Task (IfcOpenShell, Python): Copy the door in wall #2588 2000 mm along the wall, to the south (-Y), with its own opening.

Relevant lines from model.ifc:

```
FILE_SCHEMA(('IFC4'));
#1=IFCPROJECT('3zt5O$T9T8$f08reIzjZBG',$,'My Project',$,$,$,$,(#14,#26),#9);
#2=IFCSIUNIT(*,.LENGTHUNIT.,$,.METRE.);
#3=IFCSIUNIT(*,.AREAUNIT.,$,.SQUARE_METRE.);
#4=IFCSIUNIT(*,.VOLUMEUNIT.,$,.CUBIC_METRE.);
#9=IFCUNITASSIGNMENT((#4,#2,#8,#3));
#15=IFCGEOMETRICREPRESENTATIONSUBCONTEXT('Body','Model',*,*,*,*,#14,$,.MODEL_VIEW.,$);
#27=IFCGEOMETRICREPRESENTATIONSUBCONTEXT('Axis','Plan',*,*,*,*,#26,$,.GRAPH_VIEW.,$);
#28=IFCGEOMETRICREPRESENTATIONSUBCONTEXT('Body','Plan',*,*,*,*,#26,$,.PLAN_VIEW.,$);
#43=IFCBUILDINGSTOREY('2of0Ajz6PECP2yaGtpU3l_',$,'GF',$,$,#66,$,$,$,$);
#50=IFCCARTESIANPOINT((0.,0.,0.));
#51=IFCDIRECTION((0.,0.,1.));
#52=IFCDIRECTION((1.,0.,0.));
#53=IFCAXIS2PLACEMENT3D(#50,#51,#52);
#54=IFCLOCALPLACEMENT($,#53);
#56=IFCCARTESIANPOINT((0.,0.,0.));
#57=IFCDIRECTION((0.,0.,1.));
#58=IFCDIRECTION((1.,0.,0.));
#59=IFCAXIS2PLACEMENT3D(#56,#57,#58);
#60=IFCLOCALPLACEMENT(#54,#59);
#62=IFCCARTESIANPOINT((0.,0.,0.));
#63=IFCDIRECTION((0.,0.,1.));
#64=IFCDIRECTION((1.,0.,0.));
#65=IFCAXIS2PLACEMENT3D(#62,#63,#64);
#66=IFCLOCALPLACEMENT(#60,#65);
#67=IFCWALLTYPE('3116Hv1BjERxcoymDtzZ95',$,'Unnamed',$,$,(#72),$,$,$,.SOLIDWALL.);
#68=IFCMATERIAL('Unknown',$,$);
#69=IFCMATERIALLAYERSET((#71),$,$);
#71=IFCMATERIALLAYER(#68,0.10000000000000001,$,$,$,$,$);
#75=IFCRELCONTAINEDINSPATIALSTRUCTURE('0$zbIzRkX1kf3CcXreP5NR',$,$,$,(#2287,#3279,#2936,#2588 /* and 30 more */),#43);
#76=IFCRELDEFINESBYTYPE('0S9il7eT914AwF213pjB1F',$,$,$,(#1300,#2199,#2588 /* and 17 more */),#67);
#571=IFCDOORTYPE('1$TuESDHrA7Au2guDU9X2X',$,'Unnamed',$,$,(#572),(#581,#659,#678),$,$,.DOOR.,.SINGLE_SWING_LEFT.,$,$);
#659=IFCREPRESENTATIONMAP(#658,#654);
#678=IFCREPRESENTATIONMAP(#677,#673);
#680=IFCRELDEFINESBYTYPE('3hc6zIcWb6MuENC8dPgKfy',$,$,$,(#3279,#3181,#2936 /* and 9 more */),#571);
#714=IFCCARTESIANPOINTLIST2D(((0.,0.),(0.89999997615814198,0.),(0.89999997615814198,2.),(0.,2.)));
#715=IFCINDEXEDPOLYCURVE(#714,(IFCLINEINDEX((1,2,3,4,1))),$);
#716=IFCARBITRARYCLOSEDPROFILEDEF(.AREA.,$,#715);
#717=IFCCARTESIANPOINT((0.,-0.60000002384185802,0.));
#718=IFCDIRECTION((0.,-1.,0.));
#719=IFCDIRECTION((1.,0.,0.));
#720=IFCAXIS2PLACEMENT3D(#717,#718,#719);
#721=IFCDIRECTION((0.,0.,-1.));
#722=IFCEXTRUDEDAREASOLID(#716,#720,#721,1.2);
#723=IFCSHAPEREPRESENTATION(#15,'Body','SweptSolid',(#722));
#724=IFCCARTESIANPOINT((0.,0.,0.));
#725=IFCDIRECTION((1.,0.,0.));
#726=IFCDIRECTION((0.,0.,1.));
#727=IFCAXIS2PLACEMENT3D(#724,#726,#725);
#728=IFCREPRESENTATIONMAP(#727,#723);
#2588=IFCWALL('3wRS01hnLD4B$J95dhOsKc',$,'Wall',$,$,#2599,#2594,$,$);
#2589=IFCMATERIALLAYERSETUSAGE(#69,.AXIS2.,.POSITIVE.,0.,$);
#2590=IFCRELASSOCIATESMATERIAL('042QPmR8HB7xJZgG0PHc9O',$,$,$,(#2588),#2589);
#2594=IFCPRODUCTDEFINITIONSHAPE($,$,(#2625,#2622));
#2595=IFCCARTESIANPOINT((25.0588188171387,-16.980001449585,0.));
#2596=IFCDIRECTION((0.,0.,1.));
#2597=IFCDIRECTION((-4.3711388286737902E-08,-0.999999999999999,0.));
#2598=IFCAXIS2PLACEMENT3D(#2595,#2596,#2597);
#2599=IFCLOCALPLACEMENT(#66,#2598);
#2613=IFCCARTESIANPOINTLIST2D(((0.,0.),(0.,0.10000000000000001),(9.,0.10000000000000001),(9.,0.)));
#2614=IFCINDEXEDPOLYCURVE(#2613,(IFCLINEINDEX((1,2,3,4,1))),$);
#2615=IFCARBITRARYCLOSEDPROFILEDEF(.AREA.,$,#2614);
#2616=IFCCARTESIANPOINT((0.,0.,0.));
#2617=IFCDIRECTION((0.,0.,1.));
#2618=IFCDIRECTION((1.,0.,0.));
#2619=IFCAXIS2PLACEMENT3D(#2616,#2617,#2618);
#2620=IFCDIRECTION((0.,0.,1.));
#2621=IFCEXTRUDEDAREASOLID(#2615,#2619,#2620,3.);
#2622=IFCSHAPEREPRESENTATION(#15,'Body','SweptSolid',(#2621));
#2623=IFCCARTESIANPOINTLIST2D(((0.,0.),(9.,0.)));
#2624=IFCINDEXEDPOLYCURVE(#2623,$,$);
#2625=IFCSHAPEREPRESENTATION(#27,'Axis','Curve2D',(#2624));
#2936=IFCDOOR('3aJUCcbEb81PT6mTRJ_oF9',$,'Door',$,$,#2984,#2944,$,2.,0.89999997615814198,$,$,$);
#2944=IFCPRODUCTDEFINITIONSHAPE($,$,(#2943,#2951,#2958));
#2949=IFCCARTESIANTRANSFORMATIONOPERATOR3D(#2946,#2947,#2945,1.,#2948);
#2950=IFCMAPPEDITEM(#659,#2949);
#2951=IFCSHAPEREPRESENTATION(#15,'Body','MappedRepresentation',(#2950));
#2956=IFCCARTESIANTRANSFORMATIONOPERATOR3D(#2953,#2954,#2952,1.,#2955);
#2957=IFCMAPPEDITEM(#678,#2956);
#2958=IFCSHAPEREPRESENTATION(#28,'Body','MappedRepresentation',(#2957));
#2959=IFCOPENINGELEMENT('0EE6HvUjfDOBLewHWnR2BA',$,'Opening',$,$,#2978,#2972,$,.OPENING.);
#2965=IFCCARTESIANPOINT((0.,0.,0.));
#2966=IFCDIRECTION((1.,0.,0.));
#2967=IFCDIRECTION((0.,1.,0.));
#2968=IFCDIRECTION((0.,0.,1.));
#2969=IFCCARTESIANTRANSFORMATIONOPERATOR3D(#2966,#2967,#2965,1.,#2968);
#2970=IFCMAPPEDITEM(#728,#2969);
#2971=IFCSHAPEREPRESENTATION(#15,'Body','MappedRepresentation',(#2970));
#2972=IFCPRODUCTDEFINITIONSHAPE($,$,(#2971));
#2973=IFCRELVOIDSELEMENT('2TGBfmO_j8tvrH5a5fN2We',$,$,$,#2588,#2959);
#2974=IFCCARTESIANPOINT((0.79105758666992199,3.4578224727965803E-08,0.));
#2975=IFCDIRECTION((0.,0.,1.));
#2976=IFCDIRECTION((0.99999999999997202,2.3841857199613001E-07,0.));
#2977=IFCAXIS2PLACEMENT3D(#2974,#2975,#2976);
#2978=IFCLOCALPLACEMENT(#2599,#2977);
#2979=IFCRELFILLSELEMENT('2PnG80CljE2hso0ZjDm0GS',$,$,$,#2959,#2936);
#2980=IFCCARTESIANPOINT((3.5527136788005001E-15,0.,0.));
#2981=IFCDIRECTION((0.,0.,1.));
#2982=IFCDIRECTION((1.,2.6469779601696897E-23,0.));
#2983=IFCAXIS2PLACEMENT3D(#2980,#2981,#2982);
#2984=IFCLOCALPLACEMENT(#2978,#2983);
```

```python
import ifcopenshell
import ifcopenshell.api.feature
import ifcopenshell.api.geometry
import ifcopenshell.api.root
import ifcopenshell.geom
import ifcopenshell.util.element
import ifcopenshell.util.placement
import ifcopenshell.util.shape
import ifcopenshell.util.unit

model = ifcopenshell.open("model.ifc")
unit_scale = ifcopenshell.util.unit.calculate_unit_scale(model)
settings = ifcopenshell.geom.settings()


def volume(element):
    """Net volume in cubic metres, openings subtracted."""
    shape = ifcopenshell.geom.create_shape(settings, element)
    return ifcopenshell.util.shape.get_volume(shape.geometry)


door = model.by_guid("3aJUCcbEb81PT6mTRJ_oF9")
opening = door.FillsVoids[0].RelatingOpeningElement
wall = opening.VoidsElements[0].RelatingBuildingElement
before = volume(wall)
shift = ifcopenshell.util.placement.get_local_placement(wall.ObjectPlacement)[:3, 0] * 2 / unit_scale

# copy_class copies the void relationship, type, container and properties, but no geometry.
new_opening = ifcopenshell.api.root.copy_class(model, product=opening)
new_opening.Representation = ifcopenshell.util.element.copy_deep(
    model, opening.Representation, exclude=["IfcGeometricRepresentationContext", "IfcRepresentationMap"]
)
new_door = ifcopenshell.api.root.copy_class(model, product=door)
new_door.Representation = ifcopenshell.util.element.copy_deep(
    model, door.Representation, exclude=["IfcGeometricRepresentationContext", "IfcRepresentationMap"]
)
ifcopenshell.api.feature.add_filling(model, opening=new_opening, element=new_door)

for old, new in ((opening, new_opening), (door, new_door)):
    matrix = ifcopenshell.util.placement.get_local_placement(old.ObjectPlacement)
    matrix[:3, 3] += shift
    ifcopenshell.api.geometry.edit_object_placement(model, product=new, matrix=matrix, is_si=False)

after = volume(wall)

print(f"wall volume {before:.3f} -> {after:.3f} m3")

model.write("model_edited.ifc")
```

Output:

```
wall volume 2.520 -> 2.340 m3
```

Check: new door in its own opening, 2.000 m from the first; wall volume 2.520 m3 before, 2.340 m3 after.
